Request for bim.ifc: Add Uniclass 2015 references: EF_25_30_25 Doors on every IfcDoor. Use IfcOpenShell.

First a look at what the model holds.

```python
import ifcopenshell

model = ifcopenshell.open("bim.ifc")
print(model.schema)
print("classifications:", [c.Name for c in model.by_type("IfcClassification")])
for ifc_class in ("IfcDoor", "IfcRoof", "IfcStair", "IfcWall", "IfcWindow"):
    print(ifc_class, len(model.by_type(ifc_class)))
```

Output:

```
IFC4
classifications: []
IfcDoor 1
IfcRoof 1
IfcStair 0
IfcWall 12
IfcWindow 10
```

```python
import ifcopenshell
import ifcopenshell.api.classification

model = ifcopenshell.open("bim.ifc")

system = ifcopenshell.api.classification.add_classification(model, classification="Uniclass 2015")

codes = {
    "IfcDoor": ("EF_25_30_25", "Doors"),
}
for ifc_class, (code, name) in codes.items():
    products = model.by_type(ifc_class)
    ifcopenshell.api.classification.add_reference(
        model, products=products, classification=system, identification=code, name=name
    )
    print(code, len(products))

model.write("bim_edited.ifc")
```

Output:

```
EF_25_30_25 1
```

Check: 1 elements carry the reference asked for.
